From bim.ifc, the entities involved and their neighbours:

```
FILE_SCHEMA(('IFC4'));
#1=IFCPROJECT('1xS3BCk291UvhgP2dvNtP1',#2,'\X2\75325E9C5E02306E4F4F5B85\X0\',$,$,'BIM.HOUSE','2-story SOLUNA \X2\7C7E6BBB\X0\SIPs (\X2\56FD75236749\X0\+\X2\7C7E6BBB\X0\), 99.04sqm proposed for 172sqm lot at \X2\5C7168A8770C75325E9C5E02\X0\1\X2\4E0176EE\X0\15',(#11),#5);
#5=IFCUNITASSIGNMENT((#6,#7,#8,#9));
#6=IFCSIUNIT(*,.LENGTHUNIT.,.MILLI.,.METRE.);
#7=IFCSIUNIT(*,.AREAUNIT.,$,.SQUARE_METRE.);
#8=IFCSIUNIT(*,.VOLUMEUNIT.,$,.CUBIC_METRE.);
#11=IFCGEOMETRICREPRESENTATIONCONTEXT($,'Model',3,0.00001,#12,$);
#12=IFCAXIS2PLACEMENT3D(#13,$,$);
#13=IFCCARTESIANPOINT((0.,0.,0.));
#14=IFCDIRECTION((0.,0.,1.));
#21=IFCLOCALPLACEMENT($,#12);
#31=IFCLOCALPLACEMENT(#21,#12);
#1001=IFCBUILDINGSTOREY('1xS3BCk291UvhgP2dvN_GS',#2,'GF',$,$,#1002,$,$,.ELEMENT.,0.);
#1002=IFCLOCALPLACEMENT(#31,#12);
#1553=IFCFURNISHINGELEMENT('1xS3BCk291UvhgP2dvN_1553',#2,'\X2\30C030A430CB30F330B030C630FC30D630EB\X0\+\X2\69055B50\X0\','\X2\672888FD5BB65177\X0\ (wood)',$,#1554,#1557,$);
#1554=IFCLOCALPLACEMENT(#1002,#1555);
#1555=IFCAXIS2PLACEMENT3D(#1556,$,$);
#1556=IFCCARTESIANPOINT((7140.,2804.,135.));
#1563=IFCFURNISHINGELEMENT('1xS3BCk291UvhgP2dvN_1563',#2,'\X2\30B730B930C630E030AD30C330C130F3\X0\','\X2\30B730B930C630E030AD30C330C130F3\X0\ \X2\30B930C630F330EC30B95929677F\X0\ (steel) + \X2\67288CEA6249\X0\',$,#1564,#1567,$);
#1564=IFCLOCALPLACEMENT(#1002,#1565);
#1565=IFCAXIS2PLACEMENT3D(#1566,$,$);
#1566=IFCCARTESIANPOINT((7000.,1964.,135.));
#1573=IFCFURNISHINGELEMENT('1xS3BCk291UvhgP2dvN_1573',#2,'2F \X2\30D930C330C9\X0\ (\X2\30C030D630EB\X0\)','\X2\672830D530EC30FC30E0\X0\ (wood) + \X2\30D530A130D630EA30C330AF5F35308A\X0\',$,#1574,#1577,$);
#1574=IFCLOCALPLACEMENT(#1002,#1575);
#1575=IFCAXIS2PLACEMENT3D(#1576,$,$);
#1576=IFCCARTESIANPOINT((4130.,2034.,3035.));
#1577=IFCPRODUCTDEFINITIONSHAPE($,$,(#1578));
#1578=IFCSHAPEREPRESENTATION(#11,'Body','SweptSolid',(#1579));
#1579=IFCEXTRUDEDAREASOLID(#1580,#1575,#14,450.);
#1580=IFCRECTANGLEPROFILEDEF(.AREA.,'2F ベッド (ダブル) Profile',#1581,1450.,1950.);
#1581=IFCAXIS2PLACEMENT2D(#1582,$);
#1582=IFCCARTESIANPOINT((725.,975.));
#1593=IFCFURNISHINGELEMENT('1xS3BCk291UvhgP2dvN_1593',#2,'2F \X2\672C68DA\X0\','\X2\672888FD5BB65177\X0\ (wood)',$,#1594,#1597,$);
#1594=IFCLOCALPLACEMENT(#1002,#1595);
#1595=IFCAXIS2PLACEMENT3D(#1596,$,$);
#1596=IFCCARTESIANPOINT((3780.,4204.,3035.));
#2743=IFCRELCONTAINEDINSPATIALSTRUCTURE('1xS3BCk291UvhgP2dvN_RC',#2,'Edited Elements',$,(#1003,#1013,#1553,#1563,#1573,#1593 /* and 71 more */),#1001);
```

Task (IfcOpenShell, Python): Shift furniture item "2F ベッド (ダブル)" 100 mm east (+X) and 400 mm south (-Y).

```python
import ifcopenshell
import ifcopenshell.api.geometry
import ifcopenshell.util.placement

model = ifcopenshell.open("bim.ifc")

item = model.by_guid("1xS3BCk291UvhgP2dvN_1573")
matrix = ifcopenshell.util.placement.get_local_placement(item.ObjectPlacement)
matrix[0, 3] += 100.0
matrix[1, 3] -= 400.0
ifcopenshell.api.geometry.edit_object_placement(model, product=item, matrix=matrix, is_si=False)

print(ifcopenshell.util.placement.get_local_placement(item.ObjectPlacement).round(3) + 0.0)

model.write("bim_updated.ifc")
```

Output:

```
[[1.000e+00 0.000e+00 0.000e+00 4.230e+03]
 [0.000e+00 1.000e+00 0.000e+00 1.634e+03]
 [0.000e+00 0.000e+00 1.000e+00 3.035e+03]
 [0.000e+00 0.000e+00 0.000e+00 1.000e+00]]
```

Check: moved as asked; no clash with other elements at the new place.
